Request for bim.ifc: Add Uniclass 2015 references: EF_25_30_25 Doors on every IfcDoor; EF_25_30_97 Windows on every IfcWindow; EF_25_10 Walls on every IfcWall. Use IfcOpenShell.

First a look at what the model holds.

```python
import ifcopenshell

model = ifcopenshell.open("bim.ifc")
print(model.schema)
print("classifications:", [c.Name for c in model.by_type("IfcClassification")])
for ifc_class in ("IfcDoor", "IfcRoof", "IfcStair", "IfcWall", "IfcWindow"):
    print(ifc_class, len(model.by_type(ifc_class)))
```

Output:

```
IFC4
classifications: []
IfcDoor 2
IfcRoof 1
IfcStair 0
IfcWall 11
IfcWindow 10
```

```python
import ifcopenshell
import ifcopenshell.api.classification

model = ifcopenshell.open("bim.ifc")

system = ifcopenshell.api.classification.add_classification(model, classification="Uniclass 2015")

codes = {
    "IfcDoor": ("EF_25_30_25", "Doors"),
    "IfcWindow": ("EF_25_30_97", "Windows"),
    "IfcWall": ("EF_25_10", "Walls"),
}
for ifc_class, (code, name) in codes.items():
    products = model.by_type(ifc_class)
    ifcopenshell.api.classification.add_reference(
        model, products=products, classification=system, identification=code, name=name
    )
    print(code, len(products))

model.write("bim-out.ifc")
```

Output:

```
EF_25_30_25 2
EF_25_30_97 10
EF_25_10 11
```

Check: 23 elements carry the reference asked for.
